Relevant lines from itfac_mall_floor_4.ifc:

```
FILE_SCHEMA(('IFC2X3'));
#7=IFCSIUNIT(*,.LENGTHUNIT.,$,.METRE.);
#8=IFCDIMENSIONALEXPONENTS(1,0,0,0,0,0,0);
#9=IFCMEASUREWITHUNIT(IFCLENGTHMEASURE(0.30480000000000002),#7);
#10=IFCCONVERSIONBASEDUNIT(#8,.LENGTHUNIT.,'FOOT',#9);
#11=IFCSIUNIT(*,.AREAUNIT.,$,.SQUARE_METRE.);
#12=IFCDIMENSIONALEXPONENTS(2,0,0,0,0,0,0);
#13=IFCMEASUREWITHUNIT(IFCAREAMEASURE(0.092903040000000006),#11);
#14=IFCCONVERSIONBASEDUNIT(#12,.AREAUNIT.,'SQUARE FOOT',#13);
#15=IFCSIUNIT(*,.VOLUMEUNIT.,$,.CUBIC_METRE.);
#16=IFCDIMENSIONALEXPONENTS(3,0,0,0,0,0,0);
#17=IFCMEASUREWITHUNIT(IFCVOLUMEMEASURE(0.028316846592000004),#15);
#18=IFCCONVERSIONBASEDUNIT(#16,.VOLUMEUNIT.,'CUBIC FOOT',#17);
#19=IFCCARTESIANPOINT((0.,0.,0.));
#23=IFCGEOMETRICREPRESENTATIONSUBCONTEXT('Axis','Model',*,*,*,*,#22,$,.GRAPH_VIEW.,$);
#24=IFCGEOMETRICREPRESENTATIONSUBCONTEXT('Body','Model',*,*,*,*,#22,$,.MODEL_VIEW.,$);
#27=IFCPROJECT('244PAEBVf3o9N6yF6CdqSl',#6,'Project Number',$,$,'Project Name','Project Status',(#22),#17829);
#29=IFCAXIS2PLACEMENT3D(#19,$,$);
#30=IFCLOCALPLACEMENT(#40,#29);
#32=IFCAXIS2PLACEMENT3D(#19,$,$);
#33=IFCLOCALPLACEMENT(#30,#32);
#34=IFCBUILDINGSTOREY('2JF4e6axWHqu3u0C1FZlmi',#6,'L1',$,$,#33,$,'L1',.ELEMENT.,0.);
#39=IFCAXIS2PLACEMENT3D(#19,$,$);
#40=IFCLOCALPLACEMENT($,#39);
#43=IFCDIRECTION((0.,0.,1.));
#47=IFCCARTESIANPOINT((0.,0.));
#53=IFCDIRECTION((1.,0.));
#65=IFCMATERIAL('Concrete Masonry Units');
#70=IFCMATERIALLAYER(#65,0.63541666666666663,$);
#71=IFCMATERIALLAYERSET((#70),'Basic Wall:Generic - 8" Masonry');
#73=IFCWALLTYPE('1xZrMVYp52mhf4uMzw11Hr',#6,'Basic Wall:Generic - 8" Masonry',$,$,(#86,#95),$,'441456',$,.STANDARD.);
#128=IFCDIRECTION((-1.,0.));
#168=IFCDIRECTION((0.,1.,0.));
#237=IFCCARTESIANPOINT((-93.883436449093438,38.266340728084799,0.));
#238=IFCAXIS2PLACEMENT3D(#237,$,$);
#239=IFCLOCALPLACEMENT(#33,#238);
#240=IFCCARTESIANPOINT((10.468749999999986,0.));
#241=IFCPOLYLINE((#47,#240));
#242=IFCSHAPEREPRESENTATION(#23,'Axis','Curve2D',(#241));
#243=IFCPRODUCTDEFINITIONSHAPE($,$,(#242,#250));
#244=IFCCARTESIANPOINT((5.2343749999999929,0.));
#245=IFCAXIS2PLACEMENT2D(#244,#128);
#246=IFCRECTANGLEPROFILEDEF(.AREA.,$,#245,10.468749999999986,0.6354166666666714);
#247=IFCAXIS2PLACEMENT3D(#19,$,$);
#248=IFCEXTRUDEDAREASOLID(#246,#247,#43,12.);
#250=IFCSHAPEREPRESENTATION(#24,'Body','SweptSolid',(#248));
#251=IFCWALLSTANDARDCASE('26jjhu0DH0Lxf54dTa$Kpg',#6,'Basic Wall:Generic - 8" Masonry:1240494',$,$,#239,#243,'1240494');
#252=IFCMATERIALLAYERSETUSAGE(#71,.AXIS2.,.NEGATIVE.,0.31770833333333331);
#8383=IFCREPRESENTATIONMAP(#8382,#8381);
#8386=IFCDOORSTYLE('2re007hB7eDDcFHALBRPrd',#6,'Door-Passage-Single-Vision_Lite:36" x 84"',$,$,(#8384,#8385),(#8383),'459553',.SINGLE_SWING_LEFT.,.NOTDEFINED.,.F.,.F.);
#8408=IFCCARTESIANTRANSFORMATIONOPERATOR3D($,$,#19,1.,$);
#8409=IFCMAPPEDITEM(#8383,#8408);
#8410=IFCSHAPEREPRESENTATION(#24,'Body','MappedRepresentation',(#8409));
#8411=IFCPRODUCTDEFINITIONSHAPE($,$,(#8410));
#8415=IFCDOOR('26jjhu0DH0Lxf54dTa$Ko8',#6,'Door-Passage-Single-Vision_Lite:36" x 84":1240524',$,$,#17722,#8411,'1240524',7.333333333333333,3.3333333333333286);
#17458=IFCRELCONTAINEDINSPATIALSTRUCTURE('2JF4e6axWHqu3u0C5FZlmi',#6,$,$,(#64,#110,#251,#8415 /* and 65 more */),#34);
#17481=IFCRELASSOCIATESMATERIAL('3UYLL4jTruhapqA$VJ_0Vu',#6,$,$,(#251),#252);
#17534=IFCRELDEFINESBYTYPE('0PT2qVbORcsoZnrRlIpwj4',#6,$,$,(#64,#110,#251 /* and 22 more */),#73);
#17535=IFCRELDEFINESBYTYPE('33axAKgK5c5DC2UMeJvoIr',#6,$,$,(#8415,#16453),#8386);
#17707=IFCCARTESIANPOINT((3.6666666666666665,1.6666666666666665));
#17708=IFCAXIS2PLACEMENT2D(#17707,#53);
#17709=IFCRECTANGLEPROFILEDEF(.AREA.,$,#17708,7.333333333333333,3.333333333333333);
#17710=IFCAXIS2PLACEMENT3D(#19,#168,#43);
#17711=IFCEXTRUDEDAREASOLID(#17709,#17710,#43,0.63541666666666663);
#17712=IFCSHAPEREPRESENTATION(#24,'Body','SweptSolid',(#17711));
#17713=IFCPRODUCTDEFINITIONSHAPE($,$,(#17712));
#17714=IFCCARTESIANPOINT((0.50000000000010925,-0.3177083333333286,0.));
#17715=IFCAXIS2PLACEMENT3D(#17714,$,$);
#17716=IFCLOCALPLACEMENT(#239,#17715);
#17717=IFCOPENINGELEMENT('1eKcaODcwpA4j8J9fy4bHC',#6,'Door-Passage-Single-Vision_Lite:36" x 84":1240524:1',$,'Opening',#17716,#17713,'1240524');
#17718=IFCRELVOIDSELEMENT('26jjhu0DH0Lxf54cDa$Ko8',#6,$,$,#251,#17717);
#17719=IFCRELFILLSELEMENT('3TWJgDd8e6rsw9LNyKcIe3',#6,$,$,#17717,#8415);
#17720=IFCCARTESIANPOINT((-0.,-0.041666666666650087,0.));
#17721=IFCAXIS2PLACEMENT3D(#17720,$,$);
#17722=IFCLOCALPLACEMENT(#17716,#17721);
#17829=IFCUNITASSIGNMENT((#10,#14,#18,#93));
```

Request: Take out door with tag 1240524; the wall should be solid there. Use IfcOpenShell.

```python
import ifcopenshell
import ifcopenshell.api.feature
import ifcopenshell.api.root
import ifcopenshell.geom
import ifcopenshell.util.shape

model = ifcopenshell.open("itfac_mall_floor_4.ifc")
settings = ifcopenshell.geom.settings()


def volume(element):
    """Net volume in cubic metres, openings subtracted."""
    shape = ifcopenshell.geom.create_shape(settings, element)
    return ifcopenshell.util.shape.get_volume(shape.geometry)


door = model.by_id(8415)
opening = door.FillsVoids[0].RelatingOpeningElement
wall = opening.VoidsElements[0].RelatingBuildingElement
before = volume(wall)

ifcopenshell.api.root.remove_product(model, product=door)
ifcopenshell.api.feature.remove_feature(model, feature=opening)

after = volume(wall)

print(f"wall volume {before:.3f} -> {after:.3f} m3")

model.write("itfac_mall_floor_4_v2.ifc")
```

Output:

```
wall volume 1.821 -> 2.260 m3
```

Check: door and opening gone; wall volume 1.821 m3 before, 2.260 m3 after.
